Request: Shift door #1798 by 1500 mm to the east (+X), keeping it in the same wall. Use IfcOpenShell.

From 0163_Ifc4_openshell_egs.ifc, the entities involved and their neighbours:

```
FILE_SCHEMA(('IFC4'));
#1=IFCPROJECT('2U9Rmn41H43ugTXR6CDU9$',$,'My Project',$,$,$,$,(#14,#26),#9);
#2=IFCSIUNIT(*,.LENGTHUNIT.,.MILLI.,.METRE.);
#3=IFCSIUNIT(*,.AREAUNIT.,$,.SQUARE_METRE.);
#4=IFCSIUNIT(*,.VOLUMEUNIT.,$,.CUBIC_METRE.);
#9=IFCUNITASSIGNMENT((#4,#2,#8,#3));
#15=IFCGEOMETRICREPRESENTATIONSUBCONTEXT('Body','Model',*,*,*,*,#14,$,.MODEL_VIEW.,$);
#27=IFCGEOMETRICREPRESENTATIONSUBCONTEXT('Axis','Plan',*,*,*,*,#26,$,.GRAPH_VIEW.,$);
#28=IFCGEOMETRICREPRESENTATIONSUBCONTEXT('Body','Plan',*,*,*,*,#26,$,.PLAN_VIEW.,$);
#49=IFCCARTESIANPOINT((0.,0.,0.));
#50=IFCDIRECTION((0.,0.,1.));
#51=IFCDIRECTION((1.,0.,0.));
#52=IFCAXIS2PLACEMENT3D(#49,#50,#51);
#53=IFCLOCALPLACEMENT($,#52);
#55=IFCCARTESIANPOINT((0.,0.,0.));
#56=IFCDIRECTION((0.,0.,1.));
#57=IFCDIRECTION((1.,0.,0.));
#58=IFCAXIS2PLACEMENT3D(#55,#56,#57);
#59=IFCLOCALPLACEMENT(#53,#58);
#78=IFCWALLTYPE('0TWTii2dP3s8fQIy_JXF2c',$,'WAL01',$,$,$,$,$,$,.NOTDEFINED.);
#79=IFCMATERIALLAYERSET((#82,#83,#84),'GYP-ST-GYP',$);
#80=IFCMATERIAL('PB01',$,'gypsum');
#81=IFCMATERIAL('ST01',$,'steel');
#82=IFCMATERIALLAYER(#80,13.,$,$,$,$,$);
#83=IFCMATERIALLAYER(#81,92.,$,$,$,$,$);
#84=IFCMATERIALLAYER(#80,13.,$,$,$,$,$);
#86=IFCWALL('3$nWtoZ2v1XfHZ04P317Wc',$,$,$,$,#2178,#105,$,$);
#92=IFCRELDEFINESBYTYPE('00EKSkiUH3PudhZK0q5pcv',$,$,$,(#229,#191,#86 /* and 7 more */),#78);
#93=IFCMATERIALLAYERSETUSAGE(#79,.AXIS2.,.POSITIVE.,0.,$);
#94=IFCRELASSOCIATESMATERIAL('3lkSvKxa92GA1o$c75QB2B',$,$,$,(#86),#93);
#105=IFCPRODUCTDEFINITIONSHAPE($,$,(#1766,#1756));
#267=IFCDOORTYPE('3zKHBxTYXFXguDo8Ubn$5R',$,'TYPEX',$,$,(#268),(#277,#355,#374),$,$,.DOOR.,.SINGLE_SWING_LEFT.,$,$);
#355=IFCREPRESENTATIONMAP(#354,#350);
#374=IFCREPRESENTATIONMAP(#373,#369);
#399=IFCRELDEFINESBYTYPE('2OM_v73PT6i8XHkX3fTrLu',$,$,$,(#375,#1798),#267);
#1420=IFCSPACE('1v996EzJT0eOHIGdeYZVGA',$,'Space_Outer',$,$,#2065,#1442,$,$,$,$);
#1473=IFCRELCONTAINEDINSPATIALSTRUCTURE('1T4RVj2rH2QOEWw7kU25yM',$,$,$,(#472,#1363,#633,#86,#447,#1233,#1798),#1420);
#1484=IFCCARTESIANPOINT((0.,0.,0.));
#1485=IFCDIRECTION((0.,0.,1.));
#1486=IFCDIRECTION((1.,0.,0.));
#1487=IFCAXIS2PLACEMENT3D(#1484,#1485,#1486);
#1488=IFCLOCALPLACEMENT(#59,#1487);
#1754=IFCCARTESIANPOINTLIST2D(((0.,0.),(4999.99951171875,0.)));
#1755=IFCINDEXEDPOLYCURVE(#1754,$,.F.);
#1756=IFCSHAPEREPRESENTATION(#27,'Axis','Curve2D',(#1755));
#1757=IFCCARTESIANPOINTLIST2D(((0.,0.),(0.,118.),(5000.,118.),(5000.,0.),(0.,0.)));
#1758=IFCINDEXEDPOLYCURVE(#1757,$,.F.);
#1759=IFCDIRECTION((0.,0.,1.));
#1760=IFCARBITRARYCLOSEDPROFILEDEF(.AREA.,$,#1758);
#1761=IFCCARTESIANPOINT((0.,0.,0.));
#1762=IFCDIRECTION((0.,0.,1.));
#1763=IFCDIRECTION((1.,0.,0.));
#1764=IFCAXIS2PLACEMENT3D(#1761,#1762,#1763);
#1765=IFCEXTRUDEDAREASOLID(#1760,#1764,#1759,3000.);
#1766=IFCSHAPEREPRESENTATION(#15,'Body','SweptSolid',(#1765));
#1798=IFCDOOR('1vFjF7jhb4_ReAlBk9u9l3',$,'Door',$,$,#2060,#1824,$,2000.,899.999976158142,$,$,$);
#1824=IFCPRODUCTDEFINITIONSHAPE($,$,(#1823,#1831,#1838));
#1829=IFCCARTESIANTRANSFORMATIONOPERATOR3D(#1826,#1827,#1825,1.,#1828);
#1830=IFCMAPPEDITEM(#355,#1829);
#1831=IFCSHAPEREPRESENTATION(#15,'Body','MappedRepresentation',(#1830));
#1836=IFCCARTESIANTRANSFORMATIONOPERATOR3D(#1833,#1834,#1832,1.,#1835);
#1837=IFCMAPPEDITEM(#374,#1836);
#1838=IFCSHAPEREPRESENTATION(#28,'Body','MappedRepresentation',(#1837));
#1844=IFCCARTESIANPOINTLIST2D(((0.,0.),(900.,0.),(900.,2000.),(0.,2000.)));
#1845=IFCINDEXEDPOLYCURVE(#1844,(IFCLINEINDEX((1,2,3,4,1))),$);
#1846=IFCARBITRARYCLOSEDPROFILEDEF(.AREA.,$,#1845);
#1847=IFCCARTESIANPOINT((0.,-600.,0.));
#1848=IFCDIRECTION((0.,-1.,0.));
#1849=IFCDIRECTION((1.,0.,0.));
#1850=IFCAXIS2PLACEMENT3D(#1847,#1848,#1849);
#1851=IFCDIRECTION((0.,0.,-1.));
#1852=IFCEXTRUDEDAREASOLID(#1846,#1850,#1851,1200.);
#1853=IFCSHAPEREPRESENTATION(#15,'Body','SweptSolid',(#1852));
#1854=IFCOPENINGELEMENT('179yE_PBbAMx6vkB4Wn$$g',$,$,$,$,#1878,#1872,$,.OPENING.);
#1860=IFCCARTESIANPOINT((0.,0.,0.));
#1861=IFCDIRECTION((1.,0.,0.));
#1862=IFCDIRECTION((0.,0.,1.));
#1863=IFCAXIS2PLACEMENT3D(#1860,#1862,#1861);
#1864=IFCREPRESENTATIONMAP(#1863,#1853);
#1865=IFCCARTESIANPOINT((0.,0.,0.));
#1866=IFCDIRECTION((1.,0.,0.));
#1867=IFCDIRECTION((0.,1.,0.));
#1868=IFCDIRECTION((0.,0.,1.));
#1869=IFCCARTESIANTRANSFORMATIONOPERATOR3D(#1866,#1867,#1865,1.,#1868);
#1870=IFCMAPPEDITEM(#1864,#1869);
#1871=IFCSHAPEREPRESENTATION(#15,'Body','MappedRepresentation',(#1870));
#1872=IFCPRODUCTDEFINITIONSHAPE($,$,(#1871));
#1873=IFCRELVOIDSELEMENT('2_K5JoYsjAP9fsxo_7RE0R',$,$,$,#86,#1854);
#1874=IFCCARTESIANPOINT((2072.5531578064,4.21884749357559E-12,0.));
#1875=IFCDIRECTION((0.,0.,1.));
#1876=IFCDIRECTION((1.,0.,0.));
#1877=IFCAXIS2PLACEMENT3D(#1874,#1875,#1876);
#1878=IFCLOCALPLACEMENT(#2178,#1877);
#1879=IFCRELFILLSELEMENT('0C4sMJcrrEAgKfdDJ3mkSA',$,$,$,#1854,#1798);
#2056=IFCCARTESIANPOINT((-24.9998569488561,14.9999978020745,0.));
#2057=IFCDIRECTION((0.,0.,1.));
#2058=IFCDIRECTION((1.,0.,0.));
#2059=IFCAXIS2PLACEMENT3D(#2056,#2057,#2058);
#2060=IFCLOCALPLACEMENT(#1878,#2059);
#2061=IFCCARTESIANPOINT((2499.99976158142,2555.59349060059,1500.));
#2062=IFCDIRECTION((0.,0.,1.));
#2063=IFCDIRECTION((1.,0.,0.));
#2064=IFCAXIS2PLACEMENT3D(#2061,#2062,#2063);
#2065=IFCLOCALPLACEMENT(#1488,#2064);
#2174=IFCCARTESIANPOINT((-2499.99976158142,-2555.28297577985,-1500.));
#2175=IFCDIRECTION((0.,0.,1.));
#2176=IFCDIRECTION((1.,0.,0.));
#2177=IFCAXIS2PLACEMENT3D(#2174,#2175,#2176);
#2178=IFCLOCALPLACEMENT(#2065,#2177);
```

```python
import ifcopenshell
import ifcopenshell.api.geometry
import ifcopenshell.util.placement
import ifcopenshell.util.unit

model = ifcopenshell.open("0163_Ifc4_openshell_egs.ifc")
unit_scale = ifcopenshell.util.unit.calculate_unit_scale(model)

door = model.by_guid("1vFjF7jhb4_ReAlBk9u9l3")
opening = door.FillsVoids[0].RelatingOpeningElement
wall = opening.VoidsElements[0].RelatingBuildingElement

wall_matrix = ifcopenshell.util.placement.get_local_placement(wall.ObjectPlacement)
shift = wall_matrix[:3, 0] * 1.5 / unit_scale
before = ifcopenshell.util.placement.get_local_placement(door.ObjectPlacement)[:3, 3].copy()

# The door is placed relative to its opening, so it follows when the opening moves.
matrix = ifcopenshell.util.placement.get_local_placement(opening.ObjectPlacement)
matrix[:3, 3] += shift
ifcopenshell.api.geometry.edit_object_placement(
    model, product=opening, matrix=matrix, is_si=False, should_transform_children=True
)

after = ifcopenshell.util.placement.get_local_placement(door.ObjectPlacement)[:3, 3]
print("door moved by", (after - before).round(3) + 0.0)

model.write("0163_Ifc4_openshell_egs-out.ifc")
```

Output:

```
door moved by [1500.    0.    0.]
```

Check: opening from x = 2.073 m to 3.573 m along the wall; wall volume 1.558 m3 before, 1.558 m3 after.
